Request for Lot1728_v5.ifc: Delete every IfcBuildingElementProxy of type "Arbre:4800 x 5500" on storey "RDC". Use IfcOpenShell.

First a look at what the model holds.

```python
import ifcopenshell
import ifcopenshell.util.element

model = ifcopenshell.open("Lot1728_v5.ifc")
print(model.schema)
storey = next(s for s in model.by_type("IfcBuildingStorey") if s.Name == "RDC")
proxies = [e for e in ifcopenshell.util.element.get_decomposition(storey) if e.is_a("IfcBuildingElementProxy")]
seen = {}
for e in proxies:
    element_type = ifcopenshell.util.element.get_type(e)
    name = element_type.Name if element_type not in (None, e) else None
    seen[name] = seen.get(name, 0) + 1
for name, count in sorted(seen.items(), key=str):
    print(count, "x", name)
```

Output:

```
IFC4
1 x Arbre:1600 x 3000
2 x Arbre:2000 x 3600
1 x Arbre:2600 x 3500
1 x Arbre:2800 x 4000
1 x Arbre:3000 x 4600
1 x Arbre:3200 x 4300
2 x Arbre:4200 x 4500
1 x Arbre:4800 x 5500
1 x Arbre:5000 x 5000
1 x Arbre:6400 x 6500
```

```python
import ifcopenshell
import ifcopenshell.api.root
import ifcopenshell.util.element

model = ifcopenshell.open("Lot1728_v5.ifc")

storey = next(s for s in model.by_type("IfcBuildingStorey") if s.Name == "RDC")
proxies = [e for e in ifcopenshell.util.element.get_decomposition(storey) if e.is_a("IfcBuildingElementProxy")]
targets = [e for e in proxies if (t := ifcopenshell.util.element.get_type(e)) not in (None, e) and t.Name == "Arbre:4800 x 5500"]

for e in targets:
    ifcopenshell.api.root.remove_product(model, product=e)
print(len(targets), "removed")

model.write("Lot1728_v5_v2.ifc")
```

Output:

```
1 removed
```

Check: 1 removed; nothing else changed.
